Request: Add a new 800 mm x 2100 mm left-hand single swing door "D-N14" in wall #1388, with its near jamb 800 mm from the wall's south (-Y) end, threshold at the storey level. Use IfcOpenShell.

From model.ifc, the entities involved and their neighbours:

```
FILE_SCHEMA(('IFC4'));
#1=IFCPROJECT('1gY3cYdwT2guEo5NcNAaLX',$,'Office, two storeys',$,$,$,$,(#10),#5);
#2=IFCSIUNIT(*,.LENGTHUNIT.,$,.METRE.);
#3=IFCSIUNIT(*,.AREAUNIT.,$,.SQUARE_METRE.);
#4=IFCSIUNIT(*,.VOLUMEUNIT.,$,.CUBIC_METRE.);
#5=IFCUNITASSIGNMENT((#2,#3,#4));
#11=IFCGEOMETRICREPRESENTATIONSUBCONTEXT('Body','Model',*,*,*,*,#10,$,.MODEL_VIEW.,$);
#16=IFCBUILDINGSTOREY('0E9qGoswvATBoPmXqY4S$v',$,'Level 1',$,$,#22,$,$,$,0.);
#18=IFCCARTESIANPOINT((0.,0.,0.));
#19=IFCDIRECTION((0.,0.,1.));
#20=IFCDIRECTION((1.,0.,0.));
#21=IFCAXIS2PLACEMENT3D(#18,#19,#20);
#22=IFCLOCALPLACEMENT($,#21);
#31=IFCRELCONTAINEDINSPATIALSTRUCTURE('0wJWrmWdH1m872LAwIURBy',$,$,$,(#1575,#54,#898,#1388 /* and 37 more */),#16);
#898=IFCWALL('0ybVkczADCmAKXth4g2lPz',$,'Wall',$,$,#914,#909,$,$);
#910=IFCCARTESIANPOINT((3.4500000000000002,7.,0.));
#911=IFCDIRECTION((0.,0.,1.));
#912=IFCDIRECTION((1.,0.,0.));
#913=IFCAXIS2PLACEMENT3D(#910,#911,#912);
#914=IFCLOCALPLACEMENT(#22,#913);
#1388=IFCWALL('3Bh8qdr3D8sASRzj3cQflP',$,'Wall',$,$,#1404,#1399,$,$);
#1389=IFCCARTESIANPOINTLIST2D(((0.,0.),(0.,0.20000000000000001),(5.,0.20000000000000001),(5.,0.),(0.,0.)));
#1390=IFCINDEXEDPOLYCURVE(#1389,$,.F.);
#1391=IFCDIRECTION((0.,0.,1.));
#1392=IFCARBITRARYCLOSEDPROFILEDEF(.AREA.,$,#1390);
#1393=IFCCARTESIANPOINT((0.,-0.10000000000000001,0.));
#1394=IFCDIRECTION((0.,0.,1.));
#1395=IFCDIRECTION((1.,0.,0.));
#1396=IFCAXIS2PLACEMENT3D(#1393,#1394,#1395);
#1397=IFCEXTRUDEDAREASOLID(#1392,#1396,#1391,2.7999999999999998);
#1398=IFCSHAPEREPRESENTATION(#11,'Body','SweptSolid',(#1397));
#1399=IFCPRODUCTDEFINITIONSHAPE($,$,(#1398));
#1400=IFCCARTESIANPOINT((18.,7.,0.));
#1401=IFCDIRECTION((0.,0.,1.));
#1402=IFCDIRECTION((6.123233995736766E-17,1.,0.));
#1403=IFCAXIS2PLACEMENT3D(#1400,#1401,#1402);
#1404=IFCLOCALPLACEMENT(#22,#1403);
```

```python
import numpy as np
import ifcopenshell
import ifcopenshell.api.feature
import ifcopenshell.api.geometry
import ifcopenshell.api.root
import ifcopenshell.api.spatial
import ifcopenshell.geom
import ifcopenshell.util.element
import ifcopenshell.util.placement
import ifcopenshell.util.representation
import ifcopenshell.util.shape
import ifcopenshell.util.unit

model = ifcopenshell.open("model.ifc")
unit_scale = ifcopenshell.util.unit.calculate_unit_scale(model)
settings = ifcopenshell.geom.settings()


def volume(element):
    """Net volume in cubic metres, openings subtracted."""
    shape = ifcopenshell.geom.create_shape(settings, element)
    return ifcopenshell.util.shape.get_volume(shape.geometry)


wall = model.by_guid("3Bh8qdr3D8sASRzj3cQflP")
storey = ifcopenshell.util.element.get_container(wall, ifc_class="IfcBuildingStorey")
context = ifcopenshell.util.representation.get_context(model, "Model", "Body", "MODEL_VIEW")
before = volume(wall)

width, height, from_end, sill = 0.8, 2.1, 0.8, 0.0  # metres

# The wall runs along its own X axis, and the end named is its -X end.
wall_shape = ifcopenshell.geom.create_shape(settings, wall)
x, y, z = ifcopenshell.util.shape.get_vertices(wall_shape.geometry).T
start = x.min() + from_end
face, thickness = float(y.min()), float(y.max() - y.min())
wall_matrix = ifcopenshell.util.placement.get_local_placement(wall.ObjectPlacement)
level = ifcopenshell.util.placement.get_local_placement(storey.ObjectPlacement)[2, 3]


def in_wall(x, y):
    """Placement at x, y metres in the wall's axes, at sill height."""
    matrix = wall_matrix.copy()
    matrix[:, 3] = wall_matrix @ np.array([x / unit_scale, y / unit_scale, 0.0, 1.0])
    matrix[2, 3] = level + sill / unit_scale
    return matrix


# Opening: a box that overshoots both wall faces by 50 mm.
opening = ifcopenshell.api.root.create_entity(model, ifc_class="IfcOpeningElement", predefined_type="OPENING")
box = ifcopenshell.api.geometry.add_wall_representation(
    model, context=context, length=width, height=height, thickness=thickness + 0.1
)
ifcopenshell.api.geometry.assign_representation(model, product=opening, representation=box)
ifcopenshell.api.geometry.edit_object_placement(model, product=opening, matrix=in_wall(start, face - 0.05), is_si=False)
ifcopenshell.api.feature.add_feature(model, feature=opening, element=wall)

door = ifcopenshell.api.root.create_entity(model, ifc_class="IfcDoor", name="D-N14", predefined_type="DOOR")
door.OverallWidth, door.OverallHeight = width / unit_scale, height / unit_scale
door.OperationType = "SINGLE_SWING_LEFT"
body = ifcopenshell.api.geometry.add_door_representation(
    model,
    context=context,
    overall_width=door.OverallWidth,
    overall_height=door.OverallHeight,
    operation_type="SINGLE_SWING_LEFT",
    lining_properties={"LiningDepth": thickness / unit_scale, "ThresholdDepth": thickness / unit_scale},
)
ifcopenshell.api.geometry.assign_representation(model, product=door, representation=body)
ifcopenshell.api.spatial.assign_container(model, products=[door], relating_structure=storey)
ifcopenshell.api.feature.add_filling(model, opening=opening, element=door)

# The lining spans the wall, so the door starts at the wall face.
ifcopenshell.api.geometry.edit_object_placement(model, product=door, matrix=in_wall(start, face), is_si=False)

after = volume(wall)

print(f"wall volume {before:.3f} -> {after:.3f} m3")

model.write("model_edited.ifc")
```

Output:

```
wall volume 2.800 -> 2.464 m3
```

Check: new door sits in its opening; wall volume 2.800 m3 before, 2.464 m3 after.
